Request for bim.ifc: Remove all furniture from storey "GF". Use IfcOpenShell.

First a look at what the model holds.

```python
import ifcopenshell
import ifcopenshell.util.element

model = ifcopenshell.open("bim.ifc")
print(model.schema)
storey = next(s for s in model.by_type("IfcBuildingStorey") if s.Name == "GF")
furniture = [e for e in ifcopenshell.util.element.get_decomposition(storey) if e.is_a("IfcFurnishingElement")]
seen = {}
for e in furniture:
    element_type = ifcopenshell.util.element.get_type(e)
    name = element_type.Name if element_type not in (None, e) else None
    seen[name] = seen.get(name, 0) + 1
for name, count in sorted(seen.items(), key=str):
    print(count, "x", name)
```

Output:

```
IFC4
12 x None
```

```python
import ifcopenshell
import ifcopenshell.api.root
import ifcopenshell.util.element

model = ifcopenshell.open("bim.ifc")

storey = next(s for s in model.by_type("IfcBuildingStorey") if s.Name == "GF")
furniture = [e for e in ifcopenshell.util.element.get_decomposition(storey) if e.is_a("IfcFurnishingElement")]

for e in furniture:
    ifcopenshell.api.root.remove_product(model, product=e)
print(len(furniture), "removed")

model.write("bim-out.ifc")
```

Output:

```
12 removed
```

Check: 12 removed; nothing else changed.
